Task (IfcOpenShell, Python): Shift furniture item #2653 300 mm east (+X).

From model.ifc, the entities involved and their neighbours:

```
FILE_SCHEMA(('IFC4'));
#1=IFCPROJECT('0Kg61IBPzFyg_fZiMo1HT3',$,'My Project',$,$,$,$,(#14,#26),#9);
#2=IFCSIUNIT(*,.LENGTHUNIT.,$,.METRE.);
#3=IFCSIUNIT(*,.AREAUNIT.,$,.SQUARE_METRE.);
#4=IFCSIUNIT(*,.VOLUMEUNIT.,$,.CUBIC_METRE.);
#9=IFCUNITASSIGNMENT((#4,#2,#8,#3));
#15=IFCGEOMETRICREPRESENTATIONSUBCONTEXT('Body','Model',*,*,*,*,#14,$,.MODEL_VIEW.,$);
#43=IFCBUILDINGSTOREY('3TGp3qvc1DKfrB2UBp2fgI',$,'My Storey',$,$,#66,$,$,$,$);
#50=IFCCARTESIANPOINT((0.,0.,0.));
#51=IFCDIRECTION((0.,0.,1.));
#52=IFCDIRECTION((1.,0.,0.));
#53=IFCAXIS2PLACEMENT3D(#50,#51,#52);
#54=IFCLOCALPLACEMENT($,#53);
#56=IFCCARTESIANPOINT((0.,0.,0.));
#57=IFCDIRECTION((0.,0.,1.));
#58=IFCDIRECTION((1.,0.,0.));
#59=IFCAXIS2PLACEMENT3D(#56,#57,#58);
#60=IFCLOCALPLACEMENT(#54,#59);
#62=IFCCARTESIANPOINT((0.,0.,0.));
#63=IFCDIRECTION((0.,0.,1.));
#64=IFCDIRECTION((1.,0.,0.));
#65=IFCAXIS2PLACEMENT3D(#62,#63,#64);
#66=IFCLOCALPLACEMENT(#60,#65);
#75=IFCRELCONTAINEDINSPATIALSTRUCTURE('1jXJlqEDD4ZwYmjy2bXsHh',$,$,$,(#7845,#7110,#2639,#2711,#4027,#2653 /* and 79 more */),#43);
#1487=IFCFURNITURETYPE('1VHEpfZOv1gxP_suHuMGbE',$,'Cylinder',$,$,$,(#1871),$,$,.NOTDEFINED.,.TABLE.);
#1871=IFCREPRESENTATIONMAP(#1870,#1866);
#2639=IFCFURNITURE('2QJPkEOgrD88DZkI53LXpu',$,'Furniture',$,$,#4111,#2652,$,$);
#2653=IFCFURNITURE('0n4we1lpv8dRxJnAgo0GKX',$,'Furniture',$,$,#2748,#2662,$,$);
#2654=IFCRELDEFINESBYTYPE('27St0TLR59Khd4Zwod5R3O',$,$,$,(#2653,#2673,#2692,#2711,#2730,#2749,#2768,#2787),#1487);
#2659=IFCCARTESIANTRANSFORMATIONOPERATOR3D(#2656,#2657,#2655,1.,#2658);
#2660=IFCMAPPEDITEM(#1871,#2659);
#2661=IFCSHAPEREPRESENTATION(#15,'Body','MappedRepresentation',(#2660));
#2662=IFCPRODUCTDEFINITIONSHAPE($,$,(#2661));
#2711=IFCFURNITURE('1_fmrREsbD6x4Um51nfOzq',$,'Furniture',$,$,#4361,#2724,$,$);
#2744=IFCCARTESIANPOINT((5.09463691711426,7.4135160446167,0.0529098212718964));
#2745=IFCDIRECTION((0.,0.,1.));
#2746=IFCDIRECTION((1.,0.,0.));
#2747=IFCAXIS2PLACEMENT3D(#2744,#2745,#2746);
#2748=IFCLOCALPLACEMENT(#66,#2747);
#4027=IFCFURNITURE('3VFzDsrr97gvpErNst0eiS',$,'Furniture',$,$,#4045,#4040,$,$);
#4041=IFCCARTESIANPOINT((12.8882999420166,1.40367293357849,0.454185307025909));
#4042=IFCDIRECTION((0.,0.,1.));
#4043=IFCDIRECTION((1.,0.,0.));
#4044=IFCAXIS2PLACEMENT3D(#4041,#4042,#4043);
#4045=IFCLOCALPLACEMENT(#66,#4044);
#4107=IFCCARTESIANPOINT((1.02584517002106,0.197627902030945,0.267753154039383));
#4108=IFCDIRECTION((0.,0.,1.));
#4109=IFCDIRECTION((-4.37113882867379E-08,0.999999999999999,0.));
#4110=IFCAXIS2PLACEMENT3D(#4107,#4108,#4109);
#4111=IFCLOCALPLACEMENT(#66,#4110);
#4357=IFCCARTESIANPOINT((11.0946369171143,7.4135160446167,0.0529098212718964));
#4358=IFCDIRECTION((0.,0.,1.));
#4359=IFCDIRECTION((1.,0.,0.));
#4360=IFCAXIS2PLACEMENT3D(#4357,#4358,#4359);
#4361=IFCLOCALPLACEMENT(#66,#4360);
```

```python
import ifcopenshell
import ifcopenshell.api.geometry
import ifcopenshell.util.placement
import ifcopenshell.util.unit

model = ifcopenshell.open("model.ifc")
unit_scale = ifcopenshell.util.unit.calculate_unit_scale(model)

item = model.by_guid("0n4we1lpv8dRxJnAgo0GKX")
matrix = ifcopenshell.util.placement.get_local_placement(item.ObjectPlacement)
matrix[0, 3] += 0.3 / unit_scale
ifcopenshell.api.geometry.edit_object_placement(model, product=item, matrix=matrix, is_si=False)

print(ifcopenshell.util.placement.get_local_placement(item.ObjectPlacement).round(3) + 0.0)

model.write("model_edited.ifc")
```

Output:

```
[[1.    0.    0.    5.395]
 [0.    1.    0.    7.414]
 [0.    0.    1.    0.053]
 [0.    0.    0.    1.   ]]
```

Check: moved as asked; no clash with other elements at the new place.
